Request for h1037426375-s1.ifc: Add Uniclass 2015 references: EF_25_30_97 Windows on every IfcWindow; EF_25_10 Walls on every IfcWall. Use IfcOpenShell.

First a look at what the model holds.

```python
import ifcopenshell

model = ifcopenshell.open("h1037426375-s1.ifc")
print(model.schema)
print("classifications:", [c.Name for c in model.by_type("IfcClassification")])
for ifc_class in ("IfcDoor", "IfcRoof", "IfcStair", "IfcWall", "IfcWindow"):
    print(ifc_class, len(model.by_type(ifc_class)))
```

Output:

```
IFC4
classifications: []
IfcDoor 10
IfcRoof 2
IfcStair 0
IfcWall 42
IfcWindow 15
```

```python
import ifcopenshell
import ifcopenshell.api.classification

model = ifcopenshell.open("h1037426375-s1.ifc")

system = ifcopenshell.api.classification.add_classification(model, classification="Uniclass 2015")

codes = {
    "IfcWindow": ("EF_25_30_97", "Windows"),
    "IfcWall": ("EF_25_10", "Walls"),
}
for ifc_class, (code, name) in codes.items():
    products = model.by_type(ifc_class)
    ifcopenshell.api.classification.add_reference(
        model, products=products, classification=system, identification=code, name=name
    )
    print(code, len(products))

model.write("h1037426375-s1-out.ifc")
```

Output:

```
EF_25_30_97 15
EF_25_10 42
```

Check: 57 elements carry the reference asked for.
